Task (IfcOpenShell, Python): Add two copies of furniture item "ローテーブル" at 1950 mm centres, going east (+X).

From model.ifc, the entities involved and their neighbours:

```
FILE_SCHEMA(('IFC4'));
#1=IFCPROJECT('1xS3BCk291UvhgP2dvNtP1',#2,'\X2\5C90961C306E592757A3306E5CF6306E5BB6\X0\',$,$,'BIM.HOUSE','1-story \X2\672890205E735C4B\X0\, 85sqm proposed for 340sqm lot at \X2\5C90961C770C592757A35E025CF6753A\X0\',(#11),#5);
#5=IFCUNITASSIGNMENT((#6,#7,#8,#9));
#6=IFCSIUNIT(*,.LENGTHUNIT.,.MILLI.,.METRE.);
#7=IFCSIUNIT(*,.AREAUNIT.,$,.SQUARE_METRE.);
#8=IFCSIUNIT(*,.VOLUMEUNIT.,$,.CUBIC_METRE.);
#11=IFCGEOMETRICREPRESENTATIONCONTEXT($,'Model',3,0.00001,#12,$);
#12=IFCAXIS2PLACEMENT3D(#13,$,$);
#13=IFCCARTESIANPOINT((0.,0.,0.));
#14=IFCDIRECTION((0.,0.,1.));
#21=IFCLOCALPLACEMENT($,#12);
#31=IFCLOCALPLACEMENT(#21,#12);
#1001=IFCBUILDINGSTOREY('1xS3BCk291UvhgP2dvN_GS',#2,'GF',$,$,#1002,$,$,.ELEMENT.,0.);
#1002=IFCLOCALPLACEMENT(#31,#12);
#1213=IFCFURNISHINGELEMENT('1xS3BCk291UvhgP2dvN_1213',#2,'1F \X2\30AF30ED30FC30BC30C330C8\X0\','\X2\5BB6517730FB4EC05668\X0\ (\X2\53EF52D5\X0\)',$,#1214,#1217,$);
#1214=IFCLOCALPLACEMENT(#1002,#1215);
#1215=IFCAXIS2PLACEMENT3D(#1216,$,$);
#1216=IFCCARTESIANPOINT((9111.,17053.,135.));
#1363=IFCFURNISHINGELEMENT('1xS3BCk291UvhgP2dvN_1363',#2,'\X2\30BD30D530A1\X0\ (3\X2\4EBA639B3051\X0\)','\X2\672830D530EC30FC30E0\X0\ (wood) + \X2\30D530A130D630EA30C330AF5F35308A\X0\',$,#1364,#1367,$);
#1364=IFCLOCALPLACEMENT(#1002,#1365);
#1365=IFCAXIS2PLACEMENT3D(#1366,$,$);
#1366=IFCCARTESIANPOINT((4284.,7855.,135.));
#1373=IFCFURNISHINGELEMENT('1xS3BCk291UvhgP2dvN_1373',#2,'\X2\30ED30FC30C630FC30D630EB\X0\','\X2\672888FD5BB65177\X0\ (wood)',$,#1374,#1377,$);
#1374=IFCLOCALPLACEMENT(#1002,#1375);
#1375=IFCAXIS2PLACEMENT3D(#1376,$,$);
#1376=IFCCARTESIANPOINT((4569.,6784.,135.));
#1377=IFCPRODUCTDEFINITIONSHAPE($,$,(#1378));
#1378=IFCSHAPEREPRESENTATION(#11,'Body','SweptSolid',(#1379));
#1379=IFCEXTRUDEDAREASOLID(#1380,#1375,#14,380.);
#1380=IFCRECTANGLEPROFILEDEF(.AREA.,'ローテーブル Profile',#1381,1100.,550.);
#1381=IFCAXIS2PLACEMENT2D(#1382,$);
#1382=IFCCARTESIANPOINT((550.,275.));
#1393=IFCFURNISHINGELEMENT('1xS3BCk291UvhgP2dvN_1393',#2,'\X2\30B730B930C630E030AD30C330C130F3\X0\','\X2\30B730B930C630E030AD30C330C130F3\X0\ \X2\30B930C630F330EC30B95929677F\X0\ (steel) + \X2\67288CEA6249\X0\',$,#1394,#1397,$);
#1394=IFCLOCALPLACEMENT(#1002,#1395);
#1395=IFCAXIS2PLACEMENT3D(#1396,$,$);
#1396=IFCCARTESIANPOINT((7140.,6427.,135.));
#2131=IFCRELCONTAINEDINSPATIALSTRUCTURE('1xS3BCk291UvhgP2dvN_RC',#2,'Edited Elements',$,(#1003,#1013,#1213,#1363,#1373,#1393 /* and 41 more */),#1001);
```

```python
import numpy as np
import ifcopenshell
import ifcopenshell.api.geometry
import ifcopenshell.api.root
import ifcopenshell.util.element
import ifcopenshell.util.placement
import ifcopenshell.util.unit

model = ifcopenshell.open("model.ifc")
unit_scale = ifcopenshell.util.unit.calculate_unit_scale(model)


def reuse_history(source, copy):
    """copy_class also copies each property set's owner history, people and application; keep the originals."""
    for rel in copy.IsDefinedBy:
        if rel.is_a("IfcRelDefinesByProperties") and (history := rel.RelatingPropertyDefinition.OwnerHistory):
            rel.RelatingPropertyDefinition.OwnerHistory = source.OwnerHistory
            ifcopenshell.util.element.remove_deep2(model, history)


source = model.by_guid("1xS3BCk291UvhgP2dvN_1373")
base = ifcopenshell.util.placement.get_local_placement(source.ObjectPlacement)
step = np.array([1.0, 0.0, 0.0]) * 1.95 / unit_scale

for i in range(1, 3):
    copy = ifcopenshell.api.root.copy_class(model, product=source)
    copy.Representation = ifcopenshell.util.element.copy_deep(
        model, source.Representation, exclude=["IfcGeometricRepresentationContext", "IfcRepresentationMap"]
    )
    reuse_history(source, copy)
    matrix = base.copy()
    matrix[:3, 3] += i * step
    print("added at", matrix[:3, 3].round(3) + 0.0)
    ifcopenshell.api.geometry.edit_object_placement(model, product=copy, matrix=matrix, is_si=False)

model.write("model_updated.ifc")
```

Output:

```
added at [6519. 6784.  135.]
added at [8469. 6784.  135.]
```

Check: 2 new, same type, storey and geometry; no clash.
